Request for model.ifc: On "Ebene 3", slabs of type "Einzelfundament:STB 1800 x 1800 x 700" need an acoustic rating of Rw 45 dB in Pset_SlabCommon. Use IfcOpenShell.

First a look at what the model holds.

```python
import ifcopenshell
import ifcopenshell.util.element

model = ifcopenshell.open("model.ifc")
print(model.schema)
storey = next(s for s in model.by_type("IfcBuildingStorey") if s.Name == "Ebene 3")
slabs = [e for e in ifcopenshell.util.element.get_decomposition(storey) if e.is_a("IfcSlab")]
seen = {}
for e in slabs:
    element_type = ifcopenshell.util.element.get_type(e)
    key = (element_type.Name if element_type != e and element_type else None, ifcopenshell.util.element.get_pset(e, "Pset_SlabCommon", "AcousticRating"))
    seen[key] = seen.get(key, 0) + 1
for (name, value), count in sorted(seen.items(), key=str):
    print(count, "x", name, "|", value)
```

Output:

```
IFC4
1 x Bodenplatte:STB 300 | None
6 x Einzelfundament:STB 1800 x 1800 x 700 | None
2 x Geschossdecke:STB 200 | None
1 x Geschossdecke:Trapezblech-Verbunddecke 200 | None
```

```python
import ifcopenshell
import ifcopenshell.api.pset
import ifcopenshell.util.element

model = ifcopenshell.open("model.ifc")

storey = next(s for s in model.by_type("IfcBuildingStorey") if s.Name == "Ebene 3")
slabs = [e for e in ifcopenshell.util.element.get_decomposition(storey) if e.is_a("IfcSlab")]

count = 0
for e in slabs:
    element_type = ifcopenshell.util.element.get_type(e)
    if element_type in (None, e) or element_type.Name != "Einzelfundament:STB 1800 x 1800 x 700":
        continue
    # add_pset returns the element's existing set when there is one.
    pset = ifcopenshell.api.pset.add_pset(model, product=e, name="Pset_SlabCommon")
    ifcopenshell.api.pset.edit_pset(model, pset=pset, properties={"AcousticRating": "Rw 45 dB"})
    count += 1

print(count, "slabs updated")

model.write("model_updated.ifc")
```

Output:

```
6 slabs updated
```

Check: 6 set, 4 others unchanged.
